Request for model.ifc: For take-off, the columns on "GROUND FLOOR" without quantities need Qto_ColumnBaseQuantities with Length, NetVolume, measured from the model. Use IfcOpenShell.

First a look at what the model holds.

```python
import ifcopenshell
import ifcopenshell.util.element
import ifcopenshell.util.unit

model = ifcopenshell.open("model.ifc")
print(model.schema)
for unit_type in ("LENGTHUNIT", "AREAUNIT", "VOLUMEUNIT"):
    print(unit_type, ifcopenshell.util.unit.calculate_unit_scale(model, unit_type))
storey = next(s for s in model.by_type("IfcBuildingStorey") if s.Name == "GROUND FLOOR")
columns = [e for e in ifcopenshell.util.element.get_decomposition(storey) if e.is_a("IfcColumn")]
for e in sorted(columns, key=lambda e: e.id()):
    print(e.id(), e.is_a(), e.Name, list(ifcopenshell.util.element.get_psets(e, qtos_only=True)), sep=" | ")
```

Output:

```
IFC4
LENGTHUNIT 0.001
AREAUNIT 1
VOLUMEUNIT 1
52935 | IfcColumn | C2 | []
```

```python
import ifcopenshell
import ifcopenshell.api.pset
import ifcopenshell.geom
import ifcopenshell.util.element
import ifcopenshell.util.shape
import ifcopenshell.util.unit

model = ifcopenshell.open("model.ifc")
unit_scale = ifcopenshell.util.unit.calculate_unit_scale(model)
volume_scale = ifcopenshell.util.unit.calculate_unit_scale(model, "VOLUMEUNIT")
settings = ifcopenshell.geom.settings()

storey = next(s for s in model.by_type("IfcBuildingStorey") if s.Name == "GROUND FLOOR")
columns = [e for e in ifcopenshell.util.element.get_decomposition(storey) if e.is_a("IfcColumn")]

for e in sorted(columns, key=lambda e: e.id()):
    if ifcopenshell.util.element.get_psets(e, qtos_only=True, should_inherit=False):
        continue
    # Geometry comes back in metres, in the element's own axes.
    shape = ifcopenshell.geom.create_shape(settings, e)
    values = {
        "Length": ifcopenshell.util.shape.get_z(shape.geometry) / unit_scale,
        "NetVolume": ifcopenshell.util.shape.get_volume(shape.geometry) / volume_scale,
    }
    qto = ifcopenshell.api.pset.add_qto(model, product=e, name="Qto_ColumnBaseQuantities")
    ifcopenshell.api.pset.edit_qto(model, qto=qto, properties=values)
    print(e.id(), {k: round(v, 3) for k, v in values.items()})

model.write("model-out.ifc")
```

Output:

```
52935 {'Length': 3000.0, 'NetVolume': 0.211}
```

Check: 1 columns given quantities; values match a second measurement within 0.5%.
